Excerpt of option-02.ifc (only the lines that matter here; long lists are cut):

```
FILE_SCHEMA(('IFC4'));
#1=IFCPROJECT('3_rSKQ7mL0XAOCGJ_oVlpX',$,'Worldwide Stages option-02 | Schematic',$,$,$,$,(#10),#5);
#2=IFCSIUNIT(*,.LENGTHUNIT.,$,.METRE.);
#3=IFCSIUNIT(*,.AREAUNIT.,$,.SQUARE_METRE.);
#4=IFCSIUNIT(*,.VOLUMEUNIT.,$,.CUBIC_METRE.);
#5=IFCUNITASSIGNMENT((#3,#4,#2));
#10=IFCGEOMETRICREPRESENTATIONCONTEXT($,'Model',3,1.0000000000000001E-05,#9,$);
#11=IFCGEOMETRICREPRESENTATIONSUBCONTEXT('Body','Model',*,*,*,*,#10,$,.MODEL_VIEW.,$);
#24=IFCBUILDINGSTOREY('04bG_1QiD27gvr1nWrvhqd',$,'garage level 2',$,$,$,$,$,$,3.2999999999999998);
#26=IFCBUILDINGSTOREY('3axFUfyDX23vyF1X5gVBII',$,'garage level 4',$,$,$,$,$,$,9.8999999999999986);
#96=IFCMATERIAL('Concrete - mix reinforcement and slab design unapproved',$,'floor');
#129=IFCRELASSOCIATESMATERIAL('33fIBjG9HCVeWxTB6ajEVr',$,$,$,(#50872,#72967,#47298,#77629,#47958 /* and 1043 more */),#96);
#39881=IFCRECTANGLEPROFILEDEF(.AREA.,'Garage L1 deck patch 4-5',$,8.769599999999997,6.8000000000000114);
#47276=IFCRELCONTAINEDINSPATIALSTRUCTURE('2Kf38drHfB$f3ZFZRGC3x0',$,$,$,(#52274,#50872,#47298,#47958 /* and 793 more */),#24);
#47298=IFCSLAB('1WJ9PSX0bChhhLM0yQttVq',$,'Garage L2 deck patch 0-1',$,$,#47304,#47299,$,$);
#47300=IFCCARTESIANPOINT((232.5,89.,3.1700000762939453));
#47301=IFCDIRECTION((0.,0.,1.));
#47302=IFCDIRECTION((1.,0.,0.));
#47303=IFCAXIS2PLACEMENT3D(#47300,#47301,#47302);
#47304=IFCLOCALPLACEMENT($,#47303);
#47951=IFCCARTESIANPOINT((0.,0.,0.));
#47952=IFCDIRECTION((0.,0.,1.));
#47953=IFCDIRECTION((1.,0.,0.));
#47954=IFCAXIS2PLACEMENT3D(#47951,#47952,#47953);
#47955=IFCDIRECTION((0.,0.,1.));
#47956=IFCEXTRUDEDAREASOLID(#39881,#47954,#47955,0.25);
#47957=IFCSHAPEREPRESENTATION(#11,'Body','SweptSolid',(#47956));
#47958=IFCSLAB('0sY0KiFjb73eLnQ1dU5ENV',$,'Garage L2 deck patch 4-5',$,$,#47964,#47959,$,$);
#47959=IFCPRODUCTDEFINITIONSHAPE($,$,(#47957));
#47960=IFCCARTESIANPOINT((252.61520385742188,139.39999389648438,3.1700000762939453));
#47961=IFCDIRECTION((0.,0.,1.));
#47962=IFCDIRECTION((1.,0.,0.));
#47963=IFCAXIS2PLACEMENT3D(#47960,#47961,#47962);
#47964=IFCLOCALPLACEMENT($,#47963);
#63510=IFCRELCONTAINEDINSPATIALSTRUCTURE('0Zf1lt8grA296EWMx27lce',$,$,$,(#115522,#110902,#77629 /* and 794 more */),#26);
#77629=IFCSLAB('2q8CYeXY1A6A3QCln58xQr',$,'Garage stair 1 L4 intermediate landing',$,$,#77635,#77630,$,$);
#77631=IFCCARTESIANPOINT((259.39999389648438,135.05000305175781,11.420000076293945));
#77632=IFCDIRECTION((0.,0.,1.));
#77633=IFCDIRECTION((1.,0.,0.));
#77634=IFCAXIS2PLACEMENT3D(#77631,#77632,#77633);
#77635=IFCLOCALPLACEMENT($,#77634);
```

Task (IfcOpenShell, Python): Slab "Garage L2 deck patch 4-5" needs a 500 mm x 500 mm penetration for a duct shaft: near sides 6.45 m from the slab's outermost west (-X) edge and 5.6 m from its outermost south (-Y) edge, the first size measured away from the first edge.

```python
import numpy as np
import ifcopenshell
import ifcopenshell.api.feature
import ifcopenshell.api.geometry
import ifcopenshell.api.root
import ifcopenshell.geom
import ifcopenshell.util.placement
import ifcopenshell.util.representation
import ifcopenshell.util.shape
import ifcopenshell.util.unit

model = ifcopenshell.open("option-02.ifc")
unit_scale = ifcopenshell.util.unit.calculate_unit_scale(model)
settings = ifcopenshell.geom.settings()


def volume(element):
    """Net volume in cubic metres, openings subtracted."""
    shape = ifcopenshell.geom.create_shape(settings, element)
    return ifcopenshell.util.shape.get_volume(shape.geometry)


slab = model.by_id(47958)
before = volume(slab)

# Extent in the slab's own axes, in metres. The edges named are its -X and -Y sides.
slab_shape = ifcopenshell.geom.create_shape(settings, slab)
vertices = ifcopenshell.util.shape.get_vertices(slab_shape.geometry)
x_min, y_min, bottom = vertices.min(axis=0)
top = vertices[:, 2].max()

opening = ifcopenshell.api.root.create_entity(model, ifc_class="IfcOpeningElement", name="Duct shaft opening", predefined_type="OPENING")
context = ifcopenshell.util.representation.get_context(model, "Model", "Body", "MODEL_VIEW")
width, depth = 0.5, 0.5
outline = [(0.0, 0.0), (width, 0.0), (width, depth), (0.0, depth), (0.0, 0.0)]
# Overshoot both faces by 50 mm so the cut is clean.
shape = ifcopenshell.api.geometry.add_slab_representation(
    model, context=context, depth=top - bottom + 0.1, polyline=outline
)
ifcopenshell.api.geometry.assign_representation(model, product=opening, representation=shape)

matrix = ifcopenshell.util.placement.get_local_placement(slab.ObjectPlacement)
matrix[:, 3] = matrix @ np.append(np.array([x_min + 6.45, y_min + 5.6, bottom - 0.05]) / unit_scale, 1.0)
ifcopenshell.api.geometry.edit_object_placement(model, product=opening, matrix=matrix, is_si=False)
ifcopenshell.api.feature.add_feature(model, feature=opening, element=slab)

after = volume(slab)

print(f"slab volume {before:.3f} -> {after:.3f} m3")

model.write("option-02_updated.ifc")
```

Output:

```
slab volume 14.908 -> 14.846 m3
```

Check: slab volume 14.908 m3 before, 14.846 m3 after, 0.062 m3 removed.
